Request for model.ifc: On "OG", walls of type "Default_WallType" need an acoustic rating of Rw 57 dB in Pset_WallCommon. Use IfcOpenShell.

First a look at what the model holds.

```python
import ifcopenshell
import ifcopenshell.util.element

model = ifcopenshell.open("model.ifc")
print(model.schema)
storey = next(s for s in model.by_type("IfcBuildingStorey") if s.Name == "OG")
walls = [e for e in ifcopenshell.util.element.get_decomposition(storey) if e.is_a("IfcWall")]
seen = {}
for e in walls:
    element_type = ifcopenshell.util.element.get_type(e)
    key = (element_type.Name if element_type != e and element_type else None, ifcopenshell.util.element.get_pset(e, "Pset_WallCommon", "AcousticRating"))
    seen[key] = seen.get(key, 0) + 1
for (name, value), count in sorted(seen.items(), key=str):
    print(count, "x", name, "|", value)
```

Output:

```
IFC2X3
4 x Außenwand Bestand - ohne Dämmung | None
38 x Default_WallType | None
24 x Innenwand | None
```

```python
import ifcopenshell
import ifcopenshell.api.pset
import ifcopenshell.util.element

model = ifcopenshell.open("model.ifc")

storey = next(s for s in model.by_type("IfcBuildingStorey") if s.Name == "OG")
walls = [e for e in ifcopenshell.util.element.get_decomposition(storey) if e.is_a("IfcWall")]

count = 0
for e in walls:
    element_type = ifcopenshell.util.element.get_type(e)
    if element_type in (None, e) or element_type.Name != "Default_WallType":
        continue
    # add_pset returns the element's existing set when there is one.
    pset = ifcopenshell.api.pset.add_pset(model, product=e, name="Pset_WallCommon")
    ifcopenshell.api.pset.edit_pset(model, pset=pset, properties={"AcousticRating": "Rw 57 dB"})
    count += 1

print(count, "walls updated")

model.write("model_edited.ifc")
```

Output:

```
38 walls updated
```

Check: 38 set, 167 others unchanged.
